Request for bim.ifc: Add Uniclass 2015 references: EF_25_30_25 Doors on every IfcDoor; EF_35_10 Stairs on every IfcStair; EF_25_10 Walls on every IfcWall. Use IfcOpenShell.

First a look at what the model holds.

```python
import ifcopenshell

model = ifcopenshell.open("bim.ifc")
print(model.schema)
print("classifications:", [c.Name for c in model.by_type("IfcClassification")])
for ifc_class in ("IfcDoor", "IfcRoof", "IfcStair", "IfcWall", "IfcWindow"):
    print(ifc_class, len(model.by_type(ifc_class)))
```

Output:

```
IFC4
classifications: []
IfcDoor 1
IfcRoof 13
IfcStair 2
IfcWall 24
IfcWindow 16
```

```python
import ifcopenshell
import ifcopenshell.api.classification

model = ifcopenshell.open("bim.ifc")

system = ifcopenshell.api.classification.add_classification(model, classification="Uniclass 2015")

codes = {
    "IfcDoor": ("EF_25_30_25", "Doors"),
    "IfcStair": ("EF_35_10", "Stairs"),
    "IfcWall": ("EF_25_10", "Walls"),
}
for ifc_class, (code, name) in codes.items():
    products = model.by_type(ifc_class)
    ifcopenshell.api.classification.add_reference(
        model, products=products, classification=system, identification=code, name=name
    )
    print(code, len(products))

model.write("bim_rev.ifc")
```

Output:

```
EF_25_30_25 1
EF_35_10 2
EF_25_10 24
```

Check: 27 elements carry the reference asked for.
